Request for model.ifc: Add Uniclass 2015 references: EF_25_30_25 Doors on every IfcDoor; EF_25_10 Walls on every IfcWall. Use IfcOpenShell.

First a look at what the model holds.

```python
import ifcopenshell

model = ifcopenshell.open("model.ifc")
print(model.schema)
print("classifications:", [c.Name for c in model.by_type("IfcClassification")])
for ifc_class in ("IfcDoor", "IfcRoof", "IfcStair", "IfcWall", "IfcWindow"):
    print(ifc_class, len(model.by_type(ifc_class)))
```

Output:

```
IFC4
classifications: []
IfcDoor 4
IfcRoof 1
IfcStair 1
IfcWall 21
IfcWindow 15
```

```python
import ifcopenshell
import ifcopenshell.api.classification

model = ifcopenshell.open("model.ifc")

system = ifcopenshell.api.classification.add_classification(model, classification="Uniclass 2015")

codes = {
    "IfcDoor": ("EF_25_30_25", "Doors"),
    "IfcWall": ("EF_25_10", "Walls"),
}
for ifc_class, (code, name) in codes.items():
    products = model.by_type(ifc_class)
    ifcopenshell.api.classification.add_reference(
        model, products=products, classification=system, identification=code, name=name
    )
    print(code, len(products))

model.write("model-out.ifc")
```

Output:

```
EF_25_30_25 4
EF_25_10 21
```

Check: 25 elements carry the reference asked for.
